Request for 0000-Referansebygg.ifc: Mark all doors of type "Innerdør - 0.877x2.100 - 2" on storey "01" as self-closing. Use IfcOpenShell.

First a look at what the model holds.

```python
import ifcopenshell
import ifcopenshell.util.element

model = ifcopenshell.open("0000-Referansebygg.ifc")
print(model.schema)
storey = next(s for s in model.by_type("IfcBuildingStorey") if s.Name == "01")
doors = [e for e in ifcopenshell.util.element.get_decomposition(storey) if e.is_a("IfcDoor")]
seen = {}
for e in doors:
    element_type = ifcopenshell.util.element.get_type(e)
    key = (element_type.Name if element_type != e and element_type else None, ifcopenshell.util.element.get_pset(e, "Pset_DoorCommon", "SelfClosing"))
    seen[key] = seen.get(key, 0) + 1
for (name, value), count in sorted(seen.items(), key=str):
    print(count, "x", name, "|", value)
```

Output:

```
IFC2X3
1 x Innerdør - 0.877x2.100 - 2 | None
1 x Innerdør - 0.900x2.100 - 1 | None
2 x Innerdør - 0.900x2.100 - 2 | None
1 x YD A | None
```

```python
import ifcopenshell
import ifcopenshell.api.pset
import ifcopenshell.util.element

model = ifcopenshell.open("0000-Referansebygg.ifc")

storey = next(s for s in model.by_type("IfcBuildingStorey") if s.Name == "01")
doors = [e for e in ifcopenshell.util.element.get_decomposition(storey) if e.is_a("IfcDoor")]

count = 0
for e in doors:
    element_type = ifcopenshell.util.element.get_type(e)
    if element_type in (None, e) or element_type.Name != "Innerdør - 0.877x2.100 - 2":
        continue
    # add_pset returns the element's existing set when there is one.
    pset = ifcopenshell.api.pset.add_pset(model, product=e, name="Pset_DoorCommon")
    ifcopenshell.api.pset.edit_pset(model, pset=pset, properties={"SelfClosing": True})
    count += 1

print(count, "doors updated")

model.write("0000-Referansebygg_v2.ifc")
```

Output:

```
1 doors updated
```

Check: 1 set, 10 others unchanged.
